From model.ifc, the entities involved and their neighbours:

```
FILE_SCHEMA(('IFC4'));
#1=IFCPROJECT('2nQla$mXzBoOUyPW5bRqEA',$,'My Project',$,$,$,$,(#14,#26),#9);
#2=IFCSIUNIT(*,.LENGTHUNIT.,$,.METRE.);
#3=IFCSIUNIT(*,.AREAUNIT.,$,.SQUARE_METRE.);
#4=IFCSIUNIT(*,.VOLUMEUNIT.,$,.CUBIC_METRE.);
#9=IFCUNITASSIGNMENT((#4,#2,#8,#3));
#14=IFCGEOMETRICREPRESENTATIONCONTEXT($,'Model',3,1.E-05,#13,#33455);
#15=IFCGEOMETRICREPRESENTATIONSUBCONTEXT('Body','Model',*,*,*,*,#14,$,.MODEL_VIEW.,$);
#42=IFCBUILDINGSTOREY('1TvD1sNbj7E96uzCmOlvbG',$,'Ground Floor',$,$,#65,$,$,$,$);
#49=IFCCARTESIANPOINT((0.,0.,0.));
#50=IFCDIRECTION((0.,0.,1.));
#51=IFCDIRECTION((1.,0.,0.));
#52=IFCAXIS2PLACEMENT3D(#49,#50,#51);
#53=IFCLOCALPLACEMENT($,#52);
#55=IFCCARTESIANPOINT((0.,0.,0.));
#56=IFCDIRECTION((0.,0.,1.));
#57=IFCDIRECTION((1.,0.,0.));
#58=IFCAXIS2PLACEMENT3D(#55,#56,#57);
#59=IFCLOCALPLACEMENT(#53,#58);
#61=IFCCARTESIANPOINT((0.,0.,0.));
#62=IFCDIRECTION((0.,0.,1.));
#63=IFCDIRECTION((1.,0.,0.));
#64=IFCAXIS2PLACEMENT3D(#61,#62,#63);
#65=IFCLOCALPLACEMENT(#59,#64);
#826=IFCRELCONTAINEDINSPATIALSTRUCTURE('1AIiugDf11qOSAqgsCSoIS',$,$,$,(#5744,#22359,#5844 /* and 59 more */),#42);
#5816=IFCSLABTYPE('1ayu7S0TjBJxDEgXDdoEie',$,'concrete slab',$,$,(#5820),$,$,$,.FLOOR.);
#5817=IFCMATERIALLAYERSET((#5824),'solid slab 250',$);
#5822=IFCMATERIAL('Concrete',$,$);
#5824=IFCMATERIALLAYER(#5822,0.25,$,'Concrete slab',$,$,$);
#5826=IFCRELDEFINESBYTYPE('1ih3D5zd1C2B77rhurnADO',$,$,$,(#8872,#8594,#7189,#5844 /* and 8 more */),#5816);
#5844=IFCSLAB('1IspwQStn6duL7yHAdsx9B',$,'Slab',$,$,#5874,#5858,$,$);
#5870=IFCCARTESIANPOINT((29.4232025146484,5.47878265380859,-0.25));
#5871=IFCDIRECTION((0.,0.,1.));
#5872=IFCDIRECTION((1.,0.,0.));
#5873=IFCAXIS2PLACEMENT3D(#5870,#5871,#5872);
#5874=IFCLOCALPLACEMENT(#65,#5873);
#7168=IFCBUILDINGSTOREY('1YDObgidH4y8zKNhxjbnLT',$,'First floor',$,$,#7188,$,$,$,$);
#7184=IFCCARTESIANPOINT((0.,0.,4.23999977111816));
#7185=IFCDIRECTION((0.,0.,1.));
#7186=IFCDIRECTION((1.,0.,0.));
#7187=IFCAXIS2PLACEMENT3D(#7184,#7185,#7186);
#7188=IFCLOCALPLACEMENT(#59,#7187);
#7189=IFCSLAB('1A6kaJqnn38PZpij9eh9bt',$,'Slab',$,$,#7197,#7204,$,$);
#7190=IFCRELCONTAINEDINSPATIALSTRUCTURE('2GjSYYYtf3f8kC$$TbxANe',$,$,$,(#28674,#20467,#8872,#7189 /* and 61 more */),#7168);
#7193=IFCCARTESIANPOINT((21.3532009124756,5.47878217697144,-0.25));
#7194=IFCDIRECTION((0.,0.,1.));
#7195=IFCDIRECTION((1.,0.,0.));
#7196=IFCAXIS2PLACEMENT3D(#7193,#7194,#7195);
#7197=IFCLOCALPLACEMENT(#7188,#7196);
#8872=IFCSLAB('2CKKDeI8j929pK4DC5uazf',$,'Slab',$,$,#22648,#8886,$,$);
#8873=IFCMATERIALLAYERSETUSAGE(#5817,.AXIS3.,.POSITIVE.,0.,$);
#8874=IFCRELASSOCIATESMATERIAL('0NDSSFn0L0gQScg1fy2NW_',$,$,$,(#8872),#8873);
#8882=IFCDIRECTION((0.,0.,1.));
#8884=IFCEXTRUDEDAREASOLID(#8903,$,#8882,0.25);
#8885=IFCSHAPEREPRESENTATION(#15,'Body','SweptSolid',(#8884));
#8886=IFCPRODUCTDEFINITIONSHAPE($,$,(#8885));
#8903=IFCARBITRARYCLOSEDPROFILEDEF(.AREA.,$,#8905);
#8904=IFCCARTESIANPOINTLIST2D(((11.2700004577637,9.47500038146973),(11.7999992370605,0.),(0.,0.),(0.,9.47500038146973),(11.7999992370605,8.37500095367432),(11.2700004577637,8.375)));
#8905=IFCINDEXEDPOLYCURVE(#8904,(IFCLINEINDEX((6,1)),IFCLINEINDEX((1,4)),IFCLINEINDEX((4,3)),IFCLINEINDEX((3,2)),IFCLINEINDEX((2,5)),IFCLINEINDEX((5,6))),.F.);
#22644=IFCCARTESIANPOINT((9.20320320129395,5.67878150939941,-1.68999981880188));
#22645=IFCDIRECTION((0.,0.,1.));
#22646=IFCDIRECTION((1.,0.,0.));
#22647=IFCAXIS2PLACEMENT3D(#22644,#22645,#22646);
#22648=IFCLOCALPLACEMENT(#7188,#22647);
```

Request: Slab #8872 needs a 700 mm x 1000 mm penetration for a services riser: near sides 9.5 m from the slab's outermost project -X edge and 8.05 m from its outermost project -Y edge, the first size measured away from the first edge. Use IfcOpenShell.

```python
import numpy as np
import ifcopenshell
import ifcopenshell.api.feature
import ifcopenshell.api.geometry
import ifcopenshell.api.root
import ifcopenshell.geom
import ifcopenshell.util.placement
import ifcopenshell.util.representation
import ifcopenshell.util.shape
import ifcopenshell.util.unit

model = ifcopenshell.open("model.ifc")
unit_scale = ifcopenshell.util.unit.calculate_unit_scale(model)
settings = ifcopenshell.geom.settings()


def volume(element):
    """Net volume in cubic metres, openings subtracted."""
    shape = ifcopenshell.geom.create_shape(settings, element)
    return ifcopenshell.util.shape.get_volume(shape.geometry)


slab = model.by_guid("2CKKDeI8j929pK4DC5uazf")
before = volume(slab)

# Extent in the slab's own axes, in metres. The edges named are its -X and -Y sides.
slab_shape = ifcopenshell.geom.create_shape(settings, slab)
vertices = ifcopenshell.util.shape.get_vertices(slab_shape.geometry)
x_min, y_min, bottom = vertices.min(axis=0)
top = vertices[:, 2].max()

opening = ifcopenshell.api.root.create_entity(model, ifc_class="IfcOpeningElement", name="Services riser opening", predefined_type="OPENING")
context = ifcopenshell.util.representation.get_context(model, "Model", "Body", "MODEL_VIEW")
width, depth = 0.7, 1
outline = [(0.0, 0.0), (width, 0.0), (width, depth), (0.0, depth), (0.0, 0.0)]
# Overshoot both faces by 50 mm so the cut is clean.
shape = ifcopenshell.api.geometry.add_slab_representation(
    model, context=context, depth=top - bottom + 0.1, polyline=outline
)
ifcopenshell.api.geometry.assign_representation(model, product=opening, representation=shape)

matrix = ifcopenshell.util.placement.get_local_placement(slab.ObjectPlacement)
matrix[:, 3] = matrix @ np.append(np.array([x_min + 9.5, y_min + 8.05, bottom - 0.05]) / unit_scale, 1.0)
ifcopenshell.api.geometry.edit_object_placement(model, product=opening, matrix=matrix, is_si=False)
ifcopenshell.api.feature.add_feature(model, feature=opening, element=slab)

after = volume(slab)

print(f"slab volume {before:.3f} -> {after:.3f} m3")

model.write("model_rev.ifc")
```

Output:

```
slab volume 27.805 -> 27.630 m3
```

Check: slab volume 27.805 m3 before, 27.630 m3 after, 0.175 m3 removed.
